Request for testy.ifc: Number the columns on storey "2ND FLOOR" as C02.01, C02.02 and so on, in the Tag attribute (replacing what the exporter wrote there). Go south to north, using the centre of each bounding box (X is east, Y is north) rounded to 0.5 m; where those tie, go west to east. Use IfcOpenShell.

First a look at what the model holds.

```python
import ifcopenshell
import ifcopenshell.util.element
import ifcopenshell.util.placement

model = ifcopenshell.open("testy.ifc")
print(model.schema)
storey = next(s for s in model.by_type("IfcBuildingStorey") if s.Name == "2ND FLOOR")
columns = [e for e in ifcopenshell.util.element.get_decomposition(storey) if e.is_a("IfcColumn")]
for e in sorted(columns, key=lambda e: e.id()):
    origin = ifcopenshell.util.placement.get_local_placement(e.ObjectPlacement)[:3, 3]
    print(e.id(), e.Tag, e.Name, origin.round(2) + 0.0, sep=" | ")
```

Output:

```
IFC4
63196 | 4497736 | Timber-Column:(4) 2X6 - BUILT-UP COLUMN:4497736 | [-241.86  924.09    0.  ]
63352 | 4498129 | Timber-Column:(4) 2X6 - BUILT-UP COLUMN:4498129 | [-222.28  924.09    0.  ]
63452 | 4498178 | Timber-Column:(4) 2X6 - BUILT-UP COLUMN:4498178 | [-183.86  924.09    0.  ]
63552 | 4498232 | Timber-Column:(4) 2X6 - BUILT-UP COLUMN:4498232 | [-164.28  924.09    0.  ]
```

```python
import ifcopenshell
import ifcopenshell.geom
import ifcopenshell.util.element
import ifcopenshell.util.shape

model = ifcopenshell.open("testy.ifc")
settings = ifcopenshell.geom.settings()
settings.set("use-world-coords", True)


def centre(element):
    shape = ifcopenshell.geom.create_shape(settings, element)
    return ifcopenshell.util.shape.get_bbox_centroid(shape.geometry)


storey = next(s for s in model.by_type("IfcBuildingStorey") if s.Name == "2ND FLOOR")
columns = [e for e in ifcopenshell.util.element.get_decomposition(storey) if e.is_a("IfcColumn")]

# Insertion points can sit at a corner or the storey origin, so sort by the geometry (in metres).
centres = {e: centre(e) for e in columns}
columns.sort(key=lambda e: (round(centres[e][1] / 0.5), centres[e][0]))

for i, e in enumerate(columns, start=1):
    number = f"C02.{i:02d}"
    e.Tag = number
    print(e.id(), number)

model.write("testy-out.ifc")
```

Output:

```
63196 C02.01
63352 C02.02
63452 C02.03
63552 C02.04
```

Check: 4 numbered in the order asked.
